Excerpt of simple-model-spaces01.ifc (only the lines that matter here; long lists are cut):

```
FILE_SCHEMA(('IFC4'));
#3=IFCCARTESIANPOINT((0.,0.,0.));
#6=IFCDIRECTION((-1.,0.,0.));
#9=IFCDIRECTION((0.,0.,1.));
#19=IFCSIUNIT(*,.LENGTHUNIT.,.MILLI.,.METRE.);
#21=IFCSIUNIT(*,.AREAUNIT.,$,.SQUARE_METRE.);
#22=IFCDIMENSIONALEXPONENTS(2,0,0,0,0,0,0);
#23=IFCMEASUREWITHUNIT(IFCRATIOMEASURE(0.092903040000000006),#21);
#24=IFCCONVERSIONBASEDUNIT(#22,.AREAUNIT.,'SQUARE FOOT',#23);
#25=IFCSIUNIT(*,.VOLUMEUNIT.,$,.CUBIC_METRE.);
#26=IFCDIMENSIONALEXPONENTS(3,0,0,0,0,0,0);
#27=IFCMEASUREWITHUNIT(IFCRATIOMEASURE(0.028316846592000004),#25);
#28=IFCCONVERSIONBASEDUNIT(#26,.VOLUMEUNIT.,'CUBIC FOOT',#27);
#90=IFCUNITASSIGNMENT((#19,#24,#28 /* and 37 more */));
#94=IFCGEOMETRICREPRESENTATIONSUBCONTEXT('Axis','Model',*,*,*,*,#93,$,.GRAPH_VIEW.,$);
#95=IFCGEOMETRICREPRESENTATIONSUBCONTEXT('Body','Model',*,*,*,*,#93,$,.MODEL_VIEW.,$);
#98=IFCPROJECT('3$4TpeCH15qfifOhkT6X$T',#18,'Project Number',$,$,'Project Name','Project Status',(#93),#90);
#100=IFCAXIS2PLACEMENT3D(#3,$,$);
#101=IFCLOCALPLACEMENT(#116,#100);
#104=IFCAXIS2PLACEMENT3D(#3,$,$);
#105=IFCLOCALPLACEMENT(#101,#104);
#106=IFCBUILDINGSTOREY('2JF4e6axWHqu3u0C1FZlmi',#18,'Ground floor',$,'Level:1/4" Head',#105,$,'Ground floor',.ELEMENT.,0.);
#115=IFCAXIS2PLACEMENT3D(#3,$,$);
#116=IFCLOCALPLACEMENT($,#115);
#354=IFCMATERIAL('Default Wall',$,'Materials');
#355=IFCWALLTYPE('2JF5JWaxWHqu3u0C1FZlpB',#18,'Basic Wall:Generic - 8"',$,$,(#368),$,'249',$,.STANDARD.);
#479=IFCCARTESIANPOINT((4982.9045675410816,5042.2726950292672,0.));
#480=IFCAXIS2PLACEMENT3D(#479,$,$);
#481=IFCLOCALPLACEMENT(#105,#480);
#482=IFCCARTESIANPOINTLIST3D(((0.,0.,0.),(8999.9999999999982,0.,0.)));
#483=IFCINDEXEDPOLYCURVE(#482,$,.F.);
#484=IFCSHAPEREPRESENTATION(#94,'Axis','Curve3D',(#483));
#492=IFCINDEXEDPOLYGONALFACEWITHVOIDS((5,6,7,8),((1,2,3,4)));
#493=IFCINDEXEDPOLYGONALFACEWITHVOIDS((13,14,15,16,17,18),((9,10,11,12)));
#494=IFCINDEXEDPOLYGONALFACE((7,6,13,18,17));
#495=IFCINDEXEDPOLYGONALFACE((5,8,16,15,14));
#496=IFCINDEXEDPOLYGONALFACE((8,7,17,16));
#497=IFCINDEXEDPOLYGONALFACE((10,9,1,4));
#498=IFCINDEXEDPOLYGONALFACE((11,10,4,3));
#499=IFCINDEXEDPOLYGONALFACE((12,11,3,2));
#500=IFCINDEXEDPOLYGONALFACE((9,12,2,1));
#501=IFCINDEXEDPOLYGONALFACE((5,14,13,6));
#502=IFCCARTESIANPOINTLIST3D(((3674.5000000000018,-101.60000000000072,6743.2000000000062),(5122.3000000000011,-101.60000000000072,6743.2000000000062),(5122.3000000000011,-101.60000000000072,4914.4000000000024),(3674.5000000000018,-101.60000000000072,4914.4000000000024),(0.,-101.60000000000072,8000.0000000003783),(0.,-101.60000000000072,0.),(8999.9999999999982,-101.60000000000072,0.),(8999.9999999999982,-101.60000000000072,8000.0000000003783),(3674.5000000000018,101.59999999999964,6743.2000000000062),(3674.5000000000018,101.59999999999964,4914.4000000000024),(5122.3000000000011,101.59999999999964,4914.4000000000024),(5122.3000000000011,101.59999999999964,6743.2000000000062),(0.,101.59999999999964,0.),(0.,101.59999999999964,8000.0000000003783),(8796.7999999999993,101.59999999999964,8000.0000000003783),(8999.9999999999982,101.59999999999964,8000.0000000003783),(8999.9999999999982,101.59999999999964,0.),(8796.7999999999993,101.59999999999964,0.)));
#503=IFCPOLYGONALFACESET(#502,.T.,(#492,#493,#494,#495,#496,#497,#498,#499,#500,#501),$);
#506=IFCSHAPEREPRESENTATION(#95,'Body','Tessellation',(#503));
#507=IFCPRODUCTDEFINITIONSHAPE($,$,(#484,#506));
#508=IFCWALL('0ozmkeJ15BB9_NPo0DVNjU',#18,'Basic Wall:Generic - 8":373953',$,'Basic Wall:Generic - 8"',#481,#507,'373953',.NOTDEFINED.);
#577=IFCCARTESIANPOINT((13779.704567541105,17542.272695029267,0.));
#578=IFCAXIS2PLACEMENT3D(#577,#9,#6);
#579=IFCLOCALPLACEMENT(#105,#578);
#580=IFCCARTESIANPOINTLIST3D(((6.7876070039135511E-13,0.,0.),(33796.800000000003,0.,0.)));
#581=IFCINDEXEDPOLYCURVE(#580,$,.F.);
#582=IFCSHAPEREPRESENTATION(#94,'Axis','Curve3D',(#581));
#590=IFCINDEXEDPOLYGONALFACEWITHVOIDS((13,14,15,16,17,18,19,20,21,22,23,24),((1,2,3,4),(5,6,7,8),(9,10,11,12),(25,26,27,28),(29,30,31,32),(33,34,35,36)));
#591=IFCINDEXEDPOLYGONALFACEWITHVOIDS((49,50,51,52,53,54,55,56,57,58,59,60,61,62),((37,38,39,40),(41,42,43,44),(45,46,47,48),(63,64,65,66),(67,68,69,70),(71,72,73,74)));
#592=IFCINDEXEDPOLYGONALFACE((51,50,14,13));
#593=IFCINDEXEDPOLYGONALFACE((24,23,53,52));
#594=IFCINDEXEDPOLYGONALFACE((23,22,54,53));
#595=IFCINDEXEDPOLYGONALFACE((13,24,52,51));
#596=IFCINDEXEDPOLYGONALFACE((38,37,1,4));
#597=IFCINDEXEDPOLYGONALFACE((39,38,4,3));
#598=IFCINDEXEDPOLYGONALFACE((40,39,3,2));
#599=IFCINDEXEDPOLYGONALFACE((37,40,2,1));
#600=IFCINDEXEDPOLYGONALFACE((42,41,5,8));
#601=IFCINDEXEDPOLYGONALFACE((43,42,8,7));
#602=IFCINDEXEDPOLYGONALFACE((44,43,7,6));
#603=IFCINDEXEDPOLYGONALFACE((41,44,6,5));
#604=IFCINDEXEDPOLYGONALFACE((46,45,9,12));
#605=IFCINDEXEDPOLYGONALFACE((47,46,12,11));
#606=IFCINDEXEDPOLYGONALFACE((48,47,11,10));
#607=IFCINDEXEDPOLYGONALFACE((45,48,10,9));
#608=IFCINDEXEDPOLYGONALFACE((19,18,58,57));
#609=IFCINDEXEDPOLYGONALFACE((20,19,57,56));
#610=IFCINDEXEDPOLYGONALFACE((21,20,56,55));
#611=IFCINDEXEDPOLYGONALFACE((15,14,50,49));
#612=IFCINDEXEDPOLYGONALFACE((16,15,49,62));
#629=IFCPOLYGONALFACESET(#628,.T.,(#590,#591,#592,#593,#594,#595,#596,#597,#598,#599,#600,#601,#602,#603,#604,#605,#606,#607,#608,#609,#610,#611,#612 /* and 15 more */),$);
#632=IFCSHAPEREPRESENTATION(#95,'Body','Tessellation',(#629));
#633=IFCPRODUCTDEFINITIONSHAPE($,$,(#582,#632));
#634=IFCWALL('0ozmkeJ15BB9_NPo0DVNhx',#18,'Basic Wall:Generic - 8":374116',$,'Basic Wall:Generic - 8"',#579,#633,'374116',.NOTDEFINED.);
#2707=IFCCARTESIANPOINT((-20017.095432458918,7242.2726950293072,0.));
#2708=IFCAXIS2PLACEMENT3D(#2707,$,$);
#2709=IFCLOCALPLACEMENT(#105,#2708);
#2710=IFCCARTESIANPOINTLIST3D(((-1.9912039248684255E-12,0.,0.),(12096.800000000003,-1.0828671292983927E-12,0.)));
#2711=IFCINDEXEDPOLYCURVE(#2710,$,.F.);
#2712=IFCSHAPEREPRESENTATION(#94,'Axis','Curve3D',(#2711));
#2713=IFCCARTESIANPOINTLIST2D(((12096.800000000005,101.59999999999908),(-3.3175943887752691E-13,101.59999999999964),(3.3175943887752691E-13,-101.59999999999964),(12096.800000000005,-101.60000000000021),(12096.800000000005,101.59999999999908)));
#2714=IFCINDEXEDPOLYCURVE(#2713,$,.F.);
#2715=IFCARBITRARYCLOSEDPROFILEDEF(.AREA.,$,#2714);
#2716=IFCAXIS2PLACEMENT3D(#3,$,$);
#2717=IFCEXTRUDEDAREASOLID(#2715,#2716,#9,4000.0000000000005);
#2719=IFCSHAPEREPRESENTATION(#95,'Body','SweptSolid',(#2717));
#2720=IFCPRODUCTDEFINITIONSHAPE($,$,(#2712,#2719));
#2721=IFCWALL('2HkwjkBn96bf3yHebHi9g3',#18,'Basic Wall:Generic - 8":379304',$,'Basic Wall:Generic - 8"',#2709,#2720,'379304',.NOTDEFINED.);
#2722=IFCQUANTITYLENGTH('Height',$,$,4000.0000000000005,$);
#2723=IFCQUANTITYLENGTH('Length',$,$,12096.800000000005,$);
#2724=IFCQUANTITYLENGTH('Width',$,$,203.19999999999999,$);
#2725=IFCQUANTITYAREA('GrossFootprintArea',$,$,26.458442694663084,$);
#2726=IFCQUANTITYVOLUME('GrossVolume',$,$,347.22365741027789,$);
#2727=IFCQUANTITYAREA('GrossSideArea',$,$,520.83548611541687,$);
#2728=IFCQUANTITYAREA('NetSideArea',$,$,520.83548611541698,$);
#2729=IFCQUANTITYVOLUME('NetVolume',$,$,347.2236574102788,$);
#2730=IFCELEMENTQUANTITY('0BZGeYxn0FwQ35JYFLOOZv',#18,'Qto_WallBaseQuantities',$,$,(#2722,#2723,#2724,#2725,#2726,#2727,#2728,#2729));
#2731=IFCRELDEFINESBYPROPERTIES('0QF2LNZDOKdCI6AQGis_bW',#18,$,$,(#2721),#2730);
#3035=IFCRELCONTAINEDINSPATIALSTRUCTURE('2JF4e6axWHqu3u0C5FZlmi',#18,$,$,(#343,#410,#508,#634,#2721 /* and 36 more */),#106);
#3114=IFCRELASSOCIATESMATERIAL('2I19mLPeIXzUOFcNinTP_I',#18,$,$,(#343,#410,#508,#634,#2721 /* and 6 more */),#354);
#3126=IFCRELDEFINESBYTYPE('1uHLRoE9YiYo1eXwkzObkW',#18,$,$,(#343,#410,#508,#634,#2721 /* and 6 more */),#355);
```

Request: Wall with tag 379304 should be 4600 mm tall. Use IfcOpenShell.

```python
import ifcopenshell
import ifcopenshell.api.pset
import ifcopenshell.geom
import ifcopenshell.util.element
import ifcopenshell.util.representation
import ifcopenshell.util.shape
import ifcopenshell.util.unit

model = ifcopenshell.open("simple-model-spaces01.ifc")
unit_scale = ifcopenshell.util.unit.calculate_unit_scale(model)
area_scale = ifcopenshell.util.unit.calculate_unit_scale(model, "AREAUNIT")
volume_scale = ifcopenshell.util.unit.calculate_unit_scale(model, "VOLUMEUNIT")
settings = ifcopenshell.geom.settings()


def volume(element):
    """Net volume in cubic metres, openings subtracted."""
    shape = ifcopenshell.geom.create_shape(settings, element)
    return ifcopenshell.util.shape.get_volume(shape.geometry)


wall = model.by_guid("2HkwjkBn96bf3yHebHi9g3")
before = volume(wall)

body = ifcopenshell.util.representation.get_representation(wall, "Model", "Body")
solid = body.Items[0]
old_height = solid.Depth
solid.Depth = 4.6 / unit_scale
after = volume(wall)
thickness = 0.2032  # wall thickness in metres

# Update the stored height, areas and volumes.
qto = model.by_id(ifcopenshell.util.element.get_pset(wall, "Qto_WallBaseQuantities", should_inherit=False)["id"])
ifcopenshell.api.pset.edit_qto(model, qto=qto, properties={
    "Height": solid.Depth,
    "GrossVolume": ifcopenshell.util.element.get_pset(wall, "Qto_WallBaseQuantities", "GrossVolume") * solid.Depth / old_height,
    "GrossSideArea": ifcopenshell.util.element.get_pset(wall, "Qto_WallBaseQuantities", "GrossSideArea") * solid.Depth / old_height,
    "NetSideArea": after / thickness / area_scale,
    "NetVolume": after / volume_scale,
})

print(f"height {old_height:g} -> {solid.Depth:g}, volume {before:.3f} -> {after:.3f} m3")

model.write("simple-model-spaces01_v2.ifc")
```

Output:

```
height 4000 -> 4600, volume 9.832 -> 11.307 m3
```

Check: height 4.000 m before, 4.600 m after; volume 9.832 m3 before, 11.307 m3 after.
